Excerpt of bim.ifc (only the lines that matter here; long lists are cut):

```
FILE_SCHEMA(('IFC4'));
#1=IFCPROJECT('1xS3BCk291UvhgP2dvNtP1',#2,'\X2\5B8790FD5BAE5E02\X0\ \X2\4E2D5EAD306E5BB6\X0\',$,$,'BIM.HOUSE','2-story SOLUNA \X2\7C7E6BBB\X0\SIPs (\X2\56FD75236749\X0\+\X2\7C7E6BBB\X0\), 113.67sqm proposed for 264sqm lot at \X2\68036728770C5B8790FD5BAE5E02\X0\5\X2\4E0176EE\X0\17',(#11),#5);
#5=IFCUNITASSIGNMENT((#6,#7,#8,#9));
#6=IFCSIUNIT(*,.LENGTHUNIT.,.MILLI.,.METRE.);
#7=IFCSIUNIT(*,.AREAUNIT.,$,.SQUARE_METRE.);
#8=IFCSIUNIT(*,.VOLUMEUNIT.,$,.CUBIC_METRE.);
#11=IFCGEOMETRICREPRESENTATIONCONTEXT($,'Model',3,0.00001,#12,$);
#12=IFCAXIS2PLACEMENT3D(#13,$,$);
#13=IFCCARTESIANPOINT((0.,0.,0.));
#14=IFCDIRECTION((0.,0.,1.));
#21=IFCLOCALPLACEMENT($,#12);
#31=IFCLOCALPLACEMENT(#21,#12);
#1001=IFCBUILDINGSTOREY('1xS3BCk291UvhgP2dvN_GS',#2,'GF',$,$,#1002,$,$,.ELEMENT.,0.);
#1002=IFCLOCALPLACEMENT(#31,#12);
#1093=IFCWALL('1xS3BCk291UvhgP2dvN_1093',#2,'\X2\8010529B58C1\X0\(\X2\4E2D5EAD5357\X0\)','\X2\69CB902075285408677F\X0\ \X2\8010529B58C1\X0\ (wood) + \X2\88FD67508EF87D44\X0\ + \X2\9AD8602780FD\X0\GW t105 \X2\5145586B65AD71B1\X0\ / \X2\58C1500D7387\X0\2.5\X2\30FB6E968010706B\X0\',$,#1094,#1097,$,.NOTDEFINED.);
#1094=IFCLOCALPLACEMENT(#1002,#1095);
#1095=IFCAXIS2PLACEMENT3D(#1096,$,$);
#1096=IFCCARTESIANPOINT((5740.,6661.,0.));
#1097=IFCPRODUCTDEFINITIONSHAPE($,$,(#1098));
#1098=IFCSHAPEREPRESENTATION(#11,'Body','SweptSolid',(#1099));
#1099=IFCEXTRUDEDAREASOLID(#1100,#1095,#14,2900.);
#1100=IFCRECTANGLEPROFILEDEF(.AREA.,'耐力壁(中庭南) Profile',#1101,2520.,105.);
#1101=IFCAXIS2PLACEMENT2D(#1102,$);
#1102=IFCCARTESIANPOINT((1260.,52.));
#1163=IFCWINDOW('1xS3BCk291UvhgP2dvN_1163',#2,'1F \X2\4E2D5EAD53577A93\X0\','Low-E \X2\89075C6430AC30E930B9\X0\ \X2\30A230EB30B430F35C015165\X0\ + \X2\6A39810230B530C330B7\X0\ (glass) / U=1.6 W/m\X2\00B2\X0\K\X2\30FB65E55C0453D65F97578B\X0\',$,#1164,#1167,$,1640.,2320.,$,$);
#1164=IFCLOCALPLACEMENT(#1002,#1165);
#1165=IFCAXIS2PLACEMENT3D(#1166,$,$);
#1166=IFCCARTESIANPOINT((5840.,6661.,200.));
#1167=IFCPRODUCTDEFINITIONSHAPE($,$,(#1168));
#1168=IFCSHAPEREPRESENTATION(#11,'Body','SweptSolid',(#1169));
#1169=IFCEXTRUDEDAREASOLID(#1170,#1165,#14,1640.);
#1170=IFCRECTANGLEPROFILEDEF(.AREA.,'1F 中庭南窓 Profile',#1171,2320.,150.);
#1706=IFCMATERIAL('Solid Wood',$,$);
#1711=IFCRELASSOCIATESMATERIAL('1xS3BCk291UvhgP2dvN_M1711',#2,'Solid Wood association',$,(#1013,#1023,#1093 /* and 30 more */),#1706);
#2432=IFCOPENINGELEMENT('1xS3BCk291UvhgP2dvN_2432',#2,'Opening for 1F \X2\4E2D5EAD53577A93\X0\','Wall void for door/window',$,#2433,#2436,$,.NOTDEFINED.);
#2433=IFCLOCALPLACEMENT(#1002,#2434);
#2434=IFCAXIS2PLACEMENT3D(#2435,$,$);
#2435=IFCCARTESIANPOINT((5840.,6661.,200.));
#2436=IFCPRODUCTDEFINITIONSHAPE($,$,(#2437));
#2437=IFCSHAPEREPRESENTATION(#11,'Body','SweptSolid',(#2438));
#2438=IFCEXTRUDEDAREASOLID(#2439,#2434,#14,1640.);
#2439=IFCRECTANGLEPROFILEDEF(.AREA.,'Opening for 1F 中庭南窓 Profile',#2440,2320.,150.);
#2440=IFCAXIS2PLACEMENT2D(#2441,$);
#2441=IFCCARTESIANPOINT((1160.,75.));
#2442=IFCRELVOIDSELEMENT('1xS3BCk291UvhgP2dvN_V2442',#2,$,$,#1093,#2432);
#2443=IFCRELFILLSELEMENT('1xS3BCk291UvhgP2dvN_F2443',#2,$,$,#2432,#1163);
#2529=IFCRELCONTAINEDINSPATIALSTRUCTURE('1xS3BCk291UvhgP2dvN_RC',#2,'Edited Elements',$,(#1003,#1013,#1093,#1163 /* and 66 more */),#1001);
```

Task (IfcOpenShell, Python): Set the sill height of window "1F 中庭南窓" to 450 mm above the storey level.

```python
import numpy as np
import ifcopenshell
import ifcopenshell.api.geometry
import ifcopenshell.geom
import ifcopenshell.util.element
import ifcopenshell.util.placement
import ifcopenshell.util.shape
import ifcopenshell.util.unit

model = ifcopenshell.open("bim.ifc")
unit_scale = ifcopenshell.util.unit.calculate_unit_scale(model)

window = model.by_guid("1xS3BCk291UvhgP2dvN_1163")
opening = window.FillsVoids[0].RelatingOpeningElement
storey = ifcopenshell.util.element.get_container(window, ifc_class="IfcBuildingStorey")
level = ifcopenshell.util.placement.get_local_placement(storey.ObjectPlacement)[2, 3]

# The opening's origin need not be at the sill, so measure its lowest point.
shape = ifcopenshell.geom.create_shape(ifcopenshell.geom.settings(), opening)
bottom = ifcopenshell.util.shape.get_shape_bottom_elevation(shape, shape.geometry) / unit_scale
dz = level + 450.0 - bottom

shift = np.array([0.0, 0.0, dz])
# The window is not placed relative to its opening, so move both.
for product in (opening, window):
    matrix = ifcopenshell.util.placement.get_local_placement(product.ObjectPlacement)
    matrix[:3, 3] += shift
    ifcopenshell.api.geometry.edit_object_placement(model, product=product, matrix=matrix, is_si=False)

print(f"moved by {dz * unit_scale:+.3f} m")

model.write("bim_updated.ifc")
```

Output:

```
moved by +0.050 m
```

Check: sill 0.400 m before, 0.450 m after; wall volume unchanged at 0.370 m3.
